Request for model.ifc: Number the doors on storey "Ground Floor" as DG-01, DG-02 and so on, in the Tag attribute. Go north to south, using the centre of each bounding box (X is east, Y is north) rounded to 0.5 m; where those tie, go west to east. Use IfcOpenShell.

First a look at what the model holds.

```python
import ifcopenshell
import ifcopenshell.util.element
import ifcopenshell.util.placement

model = ifcopenshell.open("model.ifc")
print(model.schema)
storey = next(s for s in model.by_type("IfcBuildingStorey") if s.Name == "Ground Floor")
doors = [e for e in ifcopenshell.util.element.get_decomposition(storey) if e.is_a("IfcDoor")]
for e in sorted(doors, key=lambda e: e.id()):
    origin = ifcopenshell.util.placement.get_local_placement(e.ObjectPlacement)[:3, 3]
    print(e.id(), e.Tag, e.Name, origin.round(2) + 0.0, sep=" | ")
```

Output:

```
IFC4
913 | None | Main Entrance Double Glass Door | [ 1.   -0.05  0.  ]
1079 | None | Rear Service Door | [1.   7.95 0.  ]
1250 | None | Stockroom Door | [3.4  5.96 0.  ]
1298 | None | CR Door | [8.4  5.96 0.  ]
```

```python
import ifcopenshell
import ifcopenshell.geom
import ifcopenshell.util.element
import ifcopenshell.util.shape

model = ifcopenshell.open("model.ifc")
settings = ifcopenshell.geom.settings()
settings.set("use-world-coords", True)


def centre(element):
    shape = ifcopenshell.geom.create_shape(settings, element)
    return ifcopenshell.util.shape.get_bbox_centroid(shape.geometry)


storey = next(s for s in model.by_type("IfcBuildingStorey") if s.Name == "Ground Floor")
doors = [e for e in ifcopenshell.util.element.get_decomposition(storey) if e.is_a("IfcDoor")]

# Insertion points can sit at a corner or the storey origin, so sort by the geometry (in metres).
centres = {e: centre(e) for e in doors}
doors.sort(key=lambda e: (-round(centres[e][1] / 0.5), centres[e][0]))

for i, e in enumerate(doors, start=1):
    number = f"DG-{i:02d}"
    e.Tag = number
    print(e.id(), number)

model.write("model_v2.ifc")
```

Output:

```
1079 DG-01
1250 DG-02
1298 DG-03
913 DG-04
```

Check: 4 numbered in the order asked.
